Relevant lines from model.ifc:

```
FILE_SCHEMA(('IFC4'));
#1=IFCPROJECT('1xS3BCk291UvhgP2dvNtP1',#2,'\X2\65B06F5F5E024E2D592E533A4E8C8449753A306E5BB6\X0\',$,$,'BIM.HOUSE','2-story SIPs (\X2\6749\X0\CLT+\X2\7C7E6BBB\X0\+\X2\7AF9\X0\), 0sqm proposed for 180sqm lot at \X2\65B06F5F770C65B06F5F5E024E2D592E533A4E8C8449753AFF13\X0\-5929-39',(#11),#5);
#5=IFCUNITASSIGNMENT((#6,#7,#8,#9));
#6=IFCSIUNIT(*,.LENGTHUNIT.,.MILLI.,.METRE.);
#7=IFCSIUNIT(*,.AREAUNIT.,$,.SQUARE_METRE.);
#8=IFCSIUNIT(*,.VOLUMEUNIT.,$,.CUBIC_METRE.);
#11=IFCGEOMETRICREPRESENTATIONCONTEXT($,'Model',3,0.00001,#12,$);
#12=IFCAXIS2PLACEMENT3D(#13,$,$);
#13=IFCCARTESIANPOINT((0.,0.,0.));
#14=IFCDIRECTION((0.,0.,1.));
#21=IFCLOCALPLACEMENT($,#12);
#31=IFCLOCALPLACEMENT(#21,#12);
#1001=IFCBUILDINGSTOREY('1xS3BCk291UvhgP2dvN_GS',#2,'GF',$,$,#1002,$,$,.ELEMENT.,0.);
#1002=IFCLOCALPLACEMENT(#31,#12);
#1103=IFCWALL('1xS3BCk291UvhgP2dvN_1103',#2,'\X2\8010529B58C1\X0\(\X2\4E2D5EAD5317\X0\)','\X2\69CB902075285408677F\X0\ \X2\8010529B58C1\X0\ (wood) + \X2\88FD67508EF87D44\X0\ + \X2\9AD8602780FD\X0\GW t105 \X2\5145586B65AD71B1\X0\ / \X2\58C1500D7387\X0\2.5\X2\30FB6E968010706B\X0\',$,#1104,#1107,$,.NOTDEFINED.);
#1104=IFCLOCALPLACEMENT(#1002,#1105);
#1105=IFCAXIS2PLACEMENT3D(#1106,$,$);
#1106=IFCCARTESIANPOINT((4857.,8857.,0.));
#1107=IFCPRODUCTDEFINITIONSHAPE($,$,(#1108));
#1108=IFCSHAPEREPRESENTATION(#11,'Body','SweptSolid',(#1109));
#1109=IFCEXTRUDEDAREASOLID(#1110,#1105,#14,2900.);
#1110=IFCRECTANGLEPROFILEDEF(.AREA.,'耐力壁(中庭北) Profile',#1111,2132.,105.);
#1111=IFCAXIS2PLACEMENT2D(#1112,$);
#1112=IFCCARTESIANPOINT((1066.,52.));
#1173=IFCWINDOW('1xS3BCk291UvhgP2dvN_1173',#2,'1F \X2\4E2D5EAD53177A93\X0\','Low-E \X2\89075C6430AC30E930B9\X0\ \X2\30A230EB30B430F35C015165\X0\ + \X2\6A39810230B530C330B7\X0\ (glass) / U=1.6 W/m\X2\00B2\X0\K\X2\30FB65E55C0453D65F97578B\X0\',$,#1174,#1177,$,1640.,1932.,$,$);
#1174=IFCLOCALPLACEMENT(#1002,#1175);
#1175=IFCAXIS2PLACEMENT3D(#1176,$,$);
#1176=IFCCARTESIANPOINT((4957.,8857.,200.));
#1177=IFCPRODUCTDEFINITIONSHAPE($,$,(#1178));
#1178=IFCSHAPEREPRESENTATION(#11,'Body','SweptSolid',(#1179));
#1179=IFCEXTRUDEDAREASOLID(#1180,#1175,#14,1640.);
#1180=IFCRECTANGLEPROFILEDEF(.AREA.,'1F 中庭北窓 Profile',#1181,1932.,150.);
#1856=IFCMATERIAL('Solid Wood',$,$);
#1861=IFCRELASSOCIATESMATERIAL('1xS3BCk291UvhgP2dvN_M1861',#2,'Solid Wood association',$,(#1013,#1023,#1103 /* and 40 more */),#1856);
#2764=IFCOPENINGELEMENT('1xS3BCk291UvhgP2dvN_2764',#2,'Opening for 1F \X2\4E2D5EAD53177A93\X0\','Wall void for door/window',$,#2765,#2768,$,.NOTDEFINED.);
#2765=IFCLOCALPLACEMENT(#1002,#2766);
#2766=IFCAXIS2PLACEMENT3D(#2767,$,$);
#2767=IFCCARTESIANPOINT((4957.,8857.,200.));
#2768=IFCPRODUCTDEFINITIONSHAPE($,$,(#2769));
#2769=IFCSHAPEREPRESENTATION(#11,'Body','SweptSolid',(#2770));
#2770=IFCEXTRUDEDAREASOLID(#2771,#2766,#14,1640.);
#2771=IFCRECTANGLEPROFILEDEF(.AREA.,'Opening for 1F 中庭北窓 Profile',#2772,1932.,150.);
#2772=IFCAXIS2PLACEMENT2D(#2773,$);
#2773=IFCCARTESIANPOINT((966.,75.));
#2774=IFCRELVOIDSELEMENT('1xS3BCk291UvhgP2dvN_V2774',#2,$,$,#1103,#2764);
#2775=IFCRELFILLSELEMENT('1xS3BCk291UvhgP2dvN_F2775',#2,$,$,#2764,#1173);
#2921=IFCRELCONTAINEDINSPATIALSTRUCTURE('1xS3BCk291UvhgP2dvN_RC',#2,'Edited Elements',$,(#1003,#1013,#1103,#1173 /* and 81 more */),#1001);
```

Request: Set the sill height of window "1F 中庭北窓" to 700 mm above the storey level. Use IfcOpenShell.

```python
import numpy as np
import ifcopenshell
import ifcopenshell.api.geometry
import ifcopenshell.geom
import ifcopenshell.util.element
import ifcopenshell.util.placement
import ifcopenshell.util.shape
import ifcopenshell.util.unit

model = ifcopenshell.open("model.ifc")
unit_scale = ifcopenshell.util.unit.calculate_unit_scale(model)

window = model.by_guid("1xS3BCk291UvhgP2dvN_1173")
opening = window.FillsVoids[0].RelatingOpeningElement
storey = ifcopenshell.util.element.get_container(window, ifc_class="IfcBuildingStorey")
level = ifcopenshell.util.placement.get_local_placement(storey.ObjectPlacement)[2, 3]

# The opening's origin need not be at the sill, so measure its lowest point.
shape = ifcopenshell.geom.create_shape(ifcopenshell.geom.settings(), opening)
bottom = ifcopenshell.util.shape.get_shape_bottom_elevation(shape, shape.geometry) / unit_scale
dz = level + 0.7 / unit_scale - bottom

shift = np.array([0.0, 0.0, dz])
# The window is not placed relative to its opening, so move both.
for product in (opening, window):
    matrix = ifcopenshell.util.placement.get_local_placement(product.ObjectPlacement)
    matrix[:3, 3] += shift
    ifcopenshell.api.geometry.edit_object_placement(model, product=product, matrix=matrix, is_si=False)

print(f"moved by {dz * unit_scale:+.3f} m")

model.write("model_v2.ifc")
```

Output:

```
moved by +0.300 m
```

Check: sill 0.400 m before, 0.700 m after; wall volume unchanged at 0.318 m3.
